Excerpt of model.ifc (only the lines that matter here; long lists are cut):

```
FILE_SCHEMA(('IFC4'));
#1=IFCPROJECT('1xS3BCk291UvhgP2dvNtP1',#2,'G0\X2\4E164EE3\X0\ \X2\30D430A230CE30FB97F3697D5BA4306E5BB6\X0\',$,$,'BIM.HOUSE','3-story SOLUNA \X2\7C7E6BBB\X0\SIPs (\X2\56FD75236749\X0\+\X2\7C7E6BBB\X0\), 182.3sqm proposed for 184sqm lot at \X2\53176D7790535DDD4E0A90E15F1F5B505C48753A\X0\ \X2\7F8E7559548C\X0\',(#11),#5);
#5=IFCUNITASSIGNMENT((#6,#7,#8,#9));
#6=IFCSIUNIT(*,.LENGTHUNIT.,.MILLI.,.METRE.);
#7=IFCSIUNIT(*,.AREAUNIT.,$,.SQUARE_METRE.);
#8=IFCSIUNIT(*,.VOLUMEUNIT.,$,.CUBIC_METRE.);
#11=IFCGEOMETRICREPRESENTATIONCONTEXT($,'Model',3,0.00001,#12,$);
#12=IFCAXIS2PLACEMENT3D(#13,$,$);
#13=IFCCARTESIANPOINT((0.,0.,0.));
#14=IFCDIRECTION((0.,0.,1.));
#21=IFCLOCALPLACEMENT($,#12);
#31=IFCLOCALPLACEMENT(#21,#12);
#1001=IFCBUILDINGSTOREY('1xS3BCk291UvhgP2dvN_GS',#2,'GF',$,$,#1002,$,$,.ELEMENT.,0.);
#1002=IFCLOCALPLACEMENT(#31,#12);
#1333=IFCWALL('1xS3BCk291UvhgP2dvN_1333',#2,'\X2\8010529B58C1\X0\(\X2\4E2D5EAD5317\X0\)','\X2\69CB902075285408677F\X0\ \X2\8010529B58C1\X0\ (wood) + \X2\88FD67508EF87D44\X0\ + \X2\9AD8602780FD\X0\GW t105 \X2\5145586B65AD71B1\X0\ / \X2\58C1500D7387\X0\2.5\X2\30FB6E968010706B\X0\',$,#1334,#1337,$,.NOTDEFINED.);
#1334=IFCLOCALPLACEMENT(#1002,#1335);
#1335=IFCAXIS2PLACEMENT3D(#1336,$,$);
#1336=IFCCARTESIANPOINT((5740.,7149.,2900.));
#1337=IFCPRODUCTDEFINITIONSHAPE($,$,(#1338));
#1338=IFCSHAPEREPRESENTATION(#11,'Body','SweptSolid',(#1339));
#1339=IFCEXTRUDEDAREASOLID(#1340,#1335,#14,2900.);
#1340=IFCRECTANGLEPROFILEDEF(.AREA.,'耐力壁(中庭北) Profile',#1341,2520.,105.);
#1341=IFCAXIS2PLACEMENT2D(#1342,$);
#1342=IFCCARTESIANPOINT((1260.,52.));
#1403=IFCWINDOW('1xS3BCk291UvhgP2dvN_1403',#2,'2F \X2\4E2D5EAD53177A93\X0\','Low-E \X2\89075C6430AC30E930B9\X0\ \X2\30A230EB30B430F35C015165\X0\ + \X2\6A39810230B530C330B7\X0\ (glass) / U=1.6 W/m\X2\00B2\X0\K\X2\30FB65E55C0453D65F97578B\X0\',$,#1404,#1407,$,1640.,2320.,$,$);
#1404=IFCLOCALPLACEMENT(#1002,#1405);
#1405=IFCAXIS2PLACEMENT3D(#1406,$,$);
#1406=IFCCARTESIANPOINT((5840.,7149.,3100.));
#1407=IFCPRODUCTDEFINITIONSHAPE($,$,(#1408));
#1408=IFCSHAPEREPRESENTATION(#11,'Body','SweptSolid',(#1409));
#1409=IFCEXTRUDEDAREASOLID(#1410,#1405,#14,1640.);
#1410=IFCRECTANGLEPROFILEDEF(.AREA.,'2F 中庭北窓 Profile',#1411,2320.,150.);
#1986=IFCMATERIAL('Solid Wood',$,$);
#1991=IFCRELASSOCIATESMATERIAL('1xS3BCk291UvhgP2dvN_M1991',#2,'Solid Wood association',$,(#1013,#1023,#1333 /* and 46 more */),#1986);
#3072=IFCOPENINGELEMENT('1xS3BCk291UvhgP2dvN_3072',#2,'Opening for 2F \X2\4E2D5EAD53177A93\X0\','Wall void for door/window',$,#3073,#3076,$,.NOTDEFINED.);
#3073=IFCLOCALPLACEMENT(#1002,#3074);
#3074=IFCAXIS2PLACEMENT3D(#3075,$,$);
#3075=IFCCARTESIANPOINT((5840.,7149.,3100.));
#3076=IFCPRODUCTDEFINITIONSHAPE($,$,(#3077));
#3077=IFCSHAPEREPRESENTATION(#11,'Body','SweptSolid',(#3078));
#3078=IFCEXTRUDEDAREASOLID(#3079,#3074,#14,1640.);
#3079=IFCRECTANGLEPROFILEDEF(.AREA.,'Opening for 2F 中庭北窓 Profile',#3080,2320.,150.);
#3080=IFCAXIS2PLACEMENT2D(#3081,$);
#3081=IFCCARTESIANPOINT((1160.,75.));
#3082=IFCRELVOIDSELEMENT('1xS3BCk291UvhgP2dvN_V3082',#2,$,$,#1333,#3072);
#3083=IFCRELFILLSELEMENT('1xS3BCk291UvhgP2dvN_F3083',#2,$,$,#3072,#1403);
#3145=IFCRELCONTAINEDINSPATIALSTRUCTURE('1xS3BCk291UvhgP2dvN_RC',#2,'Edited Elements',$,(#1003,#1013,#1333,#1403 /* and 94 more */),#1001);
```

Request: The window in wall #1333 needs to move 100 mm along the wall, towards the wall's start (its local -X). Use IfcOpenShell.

```python
import ifcopenshell
import ifcopenshell.api.geometry
import ifcopenshell.util.placement
import ifcopenshell.util.unit

model = ifcopenshell.open("model.ifc")
unit_scale = ifcopenshell.util.unit.calculate_unit_scale(model)

window = model.by_guid("1xS3BCk291UvhgP2dvN_1403")
opening = window.FillsVoids[0].RelatingOpeningElement
wall = opening.VoidsElements[0].RelatingBuildingElement

wall_matrix = ifcopenshell.util.placement.get_local_placement(wall.ObjectPlacement)
shift = wall_matrix[:3, 0] * -0.1 / unit_scale
before = ifcopenshell.util.placement.get_local_placement(window.ObjectPlacement)[:3, 3].copy()

# The window is not placed relative to its opening, so move both.
for product in (opening, window):
    matrix = ifcopenshell.util.placement.get_local_placement(product.ObjectPlacement)
    matrix[:3, 3] += shift
    ifcopenshell.api.geometry.edit_object_placement(model, product=product, matrix=matrix, is_si=False)

after = ifcopenshell.util.placement.get_local_placement(window.ObjectPlacement)[:3, 3]
print("window moved by", (after - before).round(3) + 0.0)

model.write("model-out.ifc")
```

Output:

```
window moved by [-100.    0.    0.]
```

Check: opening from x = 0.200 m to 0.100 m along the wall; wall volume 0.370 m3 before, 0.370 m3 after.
